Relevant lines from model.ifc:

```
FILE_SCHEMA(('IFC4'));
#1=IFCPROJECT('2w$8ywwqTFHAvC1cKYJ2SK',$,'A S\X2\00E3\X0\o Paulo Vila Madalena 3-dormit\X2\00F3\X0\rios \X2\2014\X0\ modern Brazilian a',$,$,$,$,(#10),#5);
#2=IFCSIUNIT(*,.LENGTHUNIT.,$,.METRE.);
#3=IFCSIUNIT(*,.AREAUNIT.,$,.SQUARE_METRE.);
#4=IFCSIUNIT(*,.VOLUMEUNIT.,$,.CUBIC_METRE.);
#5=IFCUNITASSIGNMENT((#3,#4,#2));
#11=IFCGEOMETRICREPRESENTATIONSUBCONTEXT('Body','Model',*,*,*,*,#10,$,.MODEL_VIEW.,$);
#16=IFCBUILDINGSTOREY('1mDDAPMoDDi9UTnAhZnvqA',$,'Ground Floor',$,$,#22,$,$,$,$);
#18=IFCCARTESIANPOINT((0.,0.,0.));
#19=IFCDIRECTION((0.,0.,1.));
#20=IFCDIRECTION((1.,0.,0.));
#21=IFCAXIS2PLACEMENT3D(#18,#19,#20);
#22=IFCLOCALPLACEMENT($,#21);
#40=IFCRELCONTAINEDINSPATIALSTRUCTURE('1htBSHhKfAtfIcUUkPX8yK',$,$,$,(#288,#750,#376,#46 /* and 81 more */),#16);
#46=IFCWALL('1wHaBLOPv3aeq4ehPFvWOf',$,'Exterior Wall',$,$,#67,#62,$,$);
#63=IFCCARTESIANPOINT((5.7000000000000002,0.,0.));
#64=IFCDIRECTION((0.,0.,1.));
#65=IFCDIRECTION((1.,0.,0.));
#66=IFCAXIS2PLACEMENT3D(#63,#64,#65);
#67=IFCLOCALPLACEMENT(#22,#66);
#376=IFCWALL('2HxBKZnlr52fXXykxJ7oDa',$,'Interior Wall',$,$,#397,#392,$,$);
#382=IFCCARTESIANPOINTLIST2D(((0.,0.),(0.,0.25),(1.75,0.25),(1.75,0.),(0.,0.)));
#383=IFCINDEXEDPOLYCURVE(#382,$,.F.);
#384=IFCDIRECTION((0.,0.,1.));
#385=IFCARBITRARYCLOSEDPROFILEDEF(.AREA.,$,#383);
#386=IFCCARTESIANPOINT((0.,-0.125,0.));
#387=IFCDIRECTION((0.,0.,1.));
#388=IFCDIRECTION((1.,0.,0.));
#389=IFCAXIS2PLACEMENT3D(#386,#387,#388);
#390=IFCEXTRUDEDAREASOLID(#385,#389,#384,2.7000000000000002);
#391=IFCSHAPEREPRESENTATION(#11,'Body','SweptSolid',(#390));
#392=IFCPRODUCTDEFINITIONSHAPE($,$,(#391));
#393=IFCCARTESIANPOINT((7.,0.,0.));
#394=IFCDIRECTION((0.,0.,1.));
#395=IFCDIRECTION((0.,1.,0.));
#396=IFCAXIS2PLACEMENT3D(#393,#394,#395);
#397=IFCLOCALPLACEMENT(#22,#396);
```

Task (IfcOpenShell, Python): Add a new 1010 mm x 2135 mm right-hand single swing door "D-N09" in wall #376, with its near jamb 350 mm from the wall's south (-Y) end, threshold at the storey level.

```python
import numpy as np
import ifcopenshell
import ifcopenshell.api.feature
import ifcopenshell.api.geometry
import ifcopenshell.api.root
import ifcopenshell.api.spatial
import ifcopenshell.geom
import ifcopenshell.util.element
import ifcopenshell.util.placement
import ifcopenshell.util.representation
import ifcopenshell.util.shape
import ifcopenshell.util.unit

model = ifcopenshell.open("model.ifc")
unit_scale = ifcopenshell.util.unit.calculate_unit_scale(model)
settings = ifcopenshell.geom.settings()


def volume(element):
    """Net volume in cubic metres, openings subtracted."""
    shape = ifcopenshell.geom.create_shape(settings, element)
    return ifcopenshell.util.shape.get_volume(shape.geometry)


wall = model.by_guid("2HxBKZnlr52fXXykxJ7oDa")
storey = ifcopenshell.util.element.get_container(wall, ifc_class="IfcBuildingStorey")
context = ifcopenshell.util.representation.get_context(model, "Model", "Body", "MODEL_VIEW")
before = volume(wall)

width, height, from_end, sill = 1.01, 2.135, 0.35, 0.0  # metres

# The wall runs along its own X axis, and the end named is its -X end.
wall_shape = ifcopenshell.geom.create_shape(settings, wall)
x, y, z = ifcopenshell.util.shape.get_vertices(wall_shape.geometry).T
start = x.min() + from_end
face, thickness = float(y.min()), float(y.max() - y.min())
wall_matrix = ifcopenshell.util.placement.get_local_placement(wall.ObjectPlacement)
level = ifcopenshell.util.placement.get_local_placement(storey.ObjectPlacement)[2, 3]


def in_wall(x, y):
    """Placement at x, y metres in the wall's axes, at sill height."""
    matrix = wall_matrix.copy()
    matrix[:, 3] = wall_matrix @ np.array([x / unit_scale, y / unit_scale, 0.0, 1.0])
    matrix[2, 3] = level + sill / unit_scale
    return matrix


# Opening: a box that overshoots both wall faces by 50 mm.
opening = ifcopenshell.api.root.create_entity(model, ifc_class="IfcOpeningElement", predefined_type="OPENING")
box = ifcopenshell.api.geometry.add_wall_representation(
    model, context=context, length=width, height=height, thickness=thickness + 0.1
)
ifcopenshell.api.geometry.assign_representation(model, product=opening, representation=box)
ifcopenshell.api.geometry.edit_object_placement(model, product=opening, matrix=in_wall(start, face - 0.05), is_si=False)
ifcopenshell.api.feature.add_feature(model, feature=opening, element=wall)

door = ifcopenshell.api.root.create_entity(model, ifc_class="IfcDoor", name="D-N09", predefined_type="DOOR")
door.OverallWidth, door.OverallHeight = width / unit_scale, height / unit_scale
door.OperationType = "SINGLE_SWING_RIGHT"
body = ifcopenshell.api.geometry.add_door_representation(
    model,
    context=context,
    overall_width=door.OverallWidth,
    overall_height=door.OverallHeight,
    operation_type="SINGLE_SWING_RIGHT",
    lining_properties={"LiningDepth": thickness / unit_scale, "ThresholdDepth": thickness / unit_scale},
)
ifcopenshell.api.geometry.assign_representation(model, product=door, representation=body)
ifcopenshell.api.spatial.assign_container(model, products=[door], relating_structure=storey)
ifcopenshell.api.feature.add_filling(model, opening=opening, element=door)

# The lining spans the wall, so the door starts at the wall face.
ifcopenshell.api.geometry.edit_object_placement(model, product=door, matrix=in_wall(start, face), is_si=False)

after = volume(wall)

print(f"wall volume {before:.3f} -> {after:.3f} m3")

model.write("model_rev.ifc")
```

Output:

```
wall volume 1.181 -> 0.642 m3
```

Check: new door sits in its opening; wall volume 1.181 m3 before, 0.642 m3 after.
